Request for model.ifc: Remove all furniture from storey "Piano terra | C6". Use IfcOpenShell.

First a look at what the model holds.

```python
import ifcopenshell
import ifcopenshell.util.element

model = ifcopenshell.open("model.ifc")
print(model.schema)
storey = next(s for s in model.by_type("IfcBuildingStorey") if s.Name == "Piano terra | C6")
furniture = [e for e in ifcopenshell.util.element.get_decomposition(storey) if e.is_a("IfcFurnishingElement")]
seen = {}
for e in furniture:
    element_type = ifcopenshell.util.element.get_type(e)
    name = element_type.Name if element_type not in (None, e) else None
    seen[name] = seen.get(name, 0) + 1
for name, count in sorted(seen.items(), key=str):
    print(count, "x", name)
```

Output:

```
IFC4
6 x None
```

```python
import ifcopenshell
import ifcopenshell.api.root
import ifcopenshell.util.element

model = ifcopenshell.open("model.ifc")

storey = next(s for s in model.by_type("IfcBuildingStorey") if s.Name == "Piano terra | C6")
furniture = [e for e in ifcopenshell.util.element.get_decomposition(storey) if e.is_a("IfcFurnishingElement")]

for e in furniture:
    ifcopenshell.api.root.remove_product(model, product=e)
print(len(furniture), "removed")

model.write("model_edited.ifc")
```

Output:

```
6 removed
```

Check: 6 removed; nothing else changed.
